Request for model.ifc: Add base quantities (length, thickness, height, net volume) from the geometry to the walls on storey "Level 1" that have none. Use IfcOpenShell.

First a look at what the model holds.

```python
import ifcopenshell
import ifcopenshell.util.element
import ifcopenshell.util.unit

model = ifcopenshell.open("model.ifc")
print(model.schema)
for unit_type in ("LENGTHUNIT", "AREAUNIT", "VOLUMEUNIT"):
    print(unit_type, ifcopenshell.util.unit.calculate_unit_scale(model, unit_type))
storey = next(s for s in model.by_type("IfcBuildingStorey") if s.Name == "Level 1")
walls = [e for e in ifcopenshell.util.element.get_decomposition(storey) if e.is_a("IfcWall")]
for e in sorted(walls, key=lambda e: e.id()):
    print(e.id(), e.is_a(), e.Name, list(ifcopenshell.util.element.get_psets(e, qtos_only=True)), sep=" | ")
```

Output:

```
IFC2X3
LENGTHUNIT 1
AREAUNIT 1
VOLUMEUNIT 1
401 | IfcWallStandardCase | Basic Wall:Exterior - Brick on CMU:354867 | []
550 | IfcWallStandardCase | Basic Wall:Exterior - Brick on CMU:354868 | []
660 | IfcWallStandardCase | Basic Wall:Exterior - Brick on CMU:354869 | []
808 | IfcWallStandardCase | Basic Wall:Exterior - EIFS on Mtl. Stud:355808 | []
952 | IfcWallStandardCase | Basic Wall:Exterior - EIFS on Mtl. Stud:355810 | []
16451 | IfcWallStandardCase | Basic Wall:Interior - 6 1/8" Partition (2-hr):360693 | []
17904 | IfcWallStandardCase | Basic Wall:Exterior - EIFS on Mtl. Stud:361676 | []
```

```python
import ifcopenshell
import ifcopenshell.api.pset
import ifcopenshell.geom
import ifcopenshell.util.element
import ifcopenshell.util.shape
import ifcopenshell.util.unit

model = ifcopenshell.open("model.ifc")
unit_scale = ifcopenshell.util.unit.calculate_unit_scale(model)
volume_scale = ifcopenshell.util.unit.calculate_unit_scale(model, "VOLUMEUNIT")
settings = ifcopenshell.geom.settings()

storey = next(s for s in model.by_type("IfcBuildingStorey") if s.Name == "Level 1")
walls = [e for e in ifcopenshell.util.element.get_decomposition(storey) if e.is_a("IfcWall")]

for e in sorted(walls, key=lambda e: e.id()):
    if ifcopenshell.util.element.get_psets(e, qtos_only=True, should_inherit=False):
        continue
    # Geometry comes back in metres, in the element's own axes.
    shape = ifcopenshell.geom.create_shape(settings, e)
    values = {
        "Length": ifcopenshell.util.shape.get_x(shape.geometry) / unit_scale,
        "Width": ifcopenshell.util.shape.get_y(shape.geometry) / unit_scale,
        "Height": ifcopenshell.util.shape.get_z(shape.geometry) / unit_scale,
        "NetVolume": ifcopenshell.util.shape.get_volume(shape.geometry) / volume_scale,
    }
    qto = ifcopenshell.api.pset.add_qto(model, product=e, name="BaseQuantities")
    ifcopenshell.api.pset.edit_qto(model, qto=qto, properties=values)
    print(e.id(), {k: round(v, 3) for k, v in values.items()})

model.write("model_rev.ifc")
```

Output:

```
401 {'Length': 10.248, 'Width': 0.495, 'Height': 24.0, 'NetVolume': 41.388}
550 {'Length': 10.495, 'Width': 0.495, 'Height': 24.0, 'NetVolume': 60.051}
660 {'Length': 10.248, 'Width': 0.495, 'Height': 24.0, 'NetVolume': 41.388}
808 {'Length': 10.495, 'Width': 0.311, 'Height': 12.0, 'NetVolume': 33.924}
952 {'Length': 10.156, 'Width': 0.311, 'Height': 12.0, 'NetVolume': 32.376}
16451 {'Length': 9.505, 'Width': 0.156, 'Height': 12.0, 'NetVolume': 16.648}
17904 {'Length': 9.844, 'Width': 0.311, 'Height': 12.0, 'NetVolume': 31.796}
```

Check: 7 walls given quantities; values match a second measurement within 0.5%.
